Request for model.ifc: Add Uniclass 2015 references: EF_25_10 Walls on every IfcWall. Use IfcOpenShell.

First a look at what the model holds.

```python
import ifcopenshell

model = ifcopenshell.open("model.ifc")
print(model.schema)
print("classifications:", [c.Name for c in model.by_type("IfcClassification")])
for ifc_class in ("IfcDoor", "IfcRoof", "IfcStair", "IfcWall", "IfcWindow"):
    print(ifc_class, len(model.by_type(ifc_class)))
```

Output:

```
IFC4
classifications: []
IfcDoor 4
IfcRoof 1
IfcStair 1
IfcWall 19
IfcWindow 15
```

```python
import ifcopenshell
import ifcopenshell.api.classification

model = ifcopenshell.open("model.ifc")

system = ifcopenshell.api.classification.add_classification(model, classification="Uniclass 2015")

codes = {
    "IfcWall": ("EF_25_10", "Walls"),
}
for ifc_class, (code, name) in codes.items():
    products = model.by_type(ifc_class)
    ifcopenshell.api.classification.add_reference(
        model, products=products, classification=system, identification=code, name=name
    )
    print(code, len(products))

model.write("model_updated.ifc")
```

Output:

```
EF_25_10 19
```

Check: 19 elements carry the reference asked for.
